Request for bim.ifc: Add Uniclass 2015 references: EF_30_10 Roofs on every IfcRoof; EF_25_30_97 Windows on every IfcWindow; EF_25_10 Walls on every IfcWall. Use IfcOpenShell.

First a look at what the model holds.

```python
import ifcopenshell

model = ifcopenshell.open("bim.ifc")
print(model.schema)
print("classifications:", [c.Name for c in model.by_type("IfcClassification")])
for ifc_class in ("IfcDoor", "IfcRoof", "IfcStair", "IfcWall", "IfcWindow"):
    print(ifc_class, len(model.by_type(ifc_class)))
```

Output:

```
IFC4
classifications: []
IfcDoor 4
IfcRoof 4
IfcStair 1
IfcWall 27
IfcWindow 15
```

```python
import ifcopenshell
import ifcopenshell.api.classification

model = ifcopenshell.open("bim.ifc")

system = ifcopenshell.api.classification.add_classification(model, classification="Uniclass 2015")

codes = {
    "IfcRoof": ("EF_30_10", "Roofs"),
    "IfcWindow": ("EF_25_30_97", "Windows"),
    "IfcWall": ("EF_25_10", "Walls"),
}
for ifc_class, (code, name) in codes.items():
    products = model.by_type(ifc_class)
    ifcopenshell.api.classification.add_reference(
        model, products=products, classification=system, identification=code, name=name
    )
    print(code, len(products))

model.write("bim-out.ifc")
```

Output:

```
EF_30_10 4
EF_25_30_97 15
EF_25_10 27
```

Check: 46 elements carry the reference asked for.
